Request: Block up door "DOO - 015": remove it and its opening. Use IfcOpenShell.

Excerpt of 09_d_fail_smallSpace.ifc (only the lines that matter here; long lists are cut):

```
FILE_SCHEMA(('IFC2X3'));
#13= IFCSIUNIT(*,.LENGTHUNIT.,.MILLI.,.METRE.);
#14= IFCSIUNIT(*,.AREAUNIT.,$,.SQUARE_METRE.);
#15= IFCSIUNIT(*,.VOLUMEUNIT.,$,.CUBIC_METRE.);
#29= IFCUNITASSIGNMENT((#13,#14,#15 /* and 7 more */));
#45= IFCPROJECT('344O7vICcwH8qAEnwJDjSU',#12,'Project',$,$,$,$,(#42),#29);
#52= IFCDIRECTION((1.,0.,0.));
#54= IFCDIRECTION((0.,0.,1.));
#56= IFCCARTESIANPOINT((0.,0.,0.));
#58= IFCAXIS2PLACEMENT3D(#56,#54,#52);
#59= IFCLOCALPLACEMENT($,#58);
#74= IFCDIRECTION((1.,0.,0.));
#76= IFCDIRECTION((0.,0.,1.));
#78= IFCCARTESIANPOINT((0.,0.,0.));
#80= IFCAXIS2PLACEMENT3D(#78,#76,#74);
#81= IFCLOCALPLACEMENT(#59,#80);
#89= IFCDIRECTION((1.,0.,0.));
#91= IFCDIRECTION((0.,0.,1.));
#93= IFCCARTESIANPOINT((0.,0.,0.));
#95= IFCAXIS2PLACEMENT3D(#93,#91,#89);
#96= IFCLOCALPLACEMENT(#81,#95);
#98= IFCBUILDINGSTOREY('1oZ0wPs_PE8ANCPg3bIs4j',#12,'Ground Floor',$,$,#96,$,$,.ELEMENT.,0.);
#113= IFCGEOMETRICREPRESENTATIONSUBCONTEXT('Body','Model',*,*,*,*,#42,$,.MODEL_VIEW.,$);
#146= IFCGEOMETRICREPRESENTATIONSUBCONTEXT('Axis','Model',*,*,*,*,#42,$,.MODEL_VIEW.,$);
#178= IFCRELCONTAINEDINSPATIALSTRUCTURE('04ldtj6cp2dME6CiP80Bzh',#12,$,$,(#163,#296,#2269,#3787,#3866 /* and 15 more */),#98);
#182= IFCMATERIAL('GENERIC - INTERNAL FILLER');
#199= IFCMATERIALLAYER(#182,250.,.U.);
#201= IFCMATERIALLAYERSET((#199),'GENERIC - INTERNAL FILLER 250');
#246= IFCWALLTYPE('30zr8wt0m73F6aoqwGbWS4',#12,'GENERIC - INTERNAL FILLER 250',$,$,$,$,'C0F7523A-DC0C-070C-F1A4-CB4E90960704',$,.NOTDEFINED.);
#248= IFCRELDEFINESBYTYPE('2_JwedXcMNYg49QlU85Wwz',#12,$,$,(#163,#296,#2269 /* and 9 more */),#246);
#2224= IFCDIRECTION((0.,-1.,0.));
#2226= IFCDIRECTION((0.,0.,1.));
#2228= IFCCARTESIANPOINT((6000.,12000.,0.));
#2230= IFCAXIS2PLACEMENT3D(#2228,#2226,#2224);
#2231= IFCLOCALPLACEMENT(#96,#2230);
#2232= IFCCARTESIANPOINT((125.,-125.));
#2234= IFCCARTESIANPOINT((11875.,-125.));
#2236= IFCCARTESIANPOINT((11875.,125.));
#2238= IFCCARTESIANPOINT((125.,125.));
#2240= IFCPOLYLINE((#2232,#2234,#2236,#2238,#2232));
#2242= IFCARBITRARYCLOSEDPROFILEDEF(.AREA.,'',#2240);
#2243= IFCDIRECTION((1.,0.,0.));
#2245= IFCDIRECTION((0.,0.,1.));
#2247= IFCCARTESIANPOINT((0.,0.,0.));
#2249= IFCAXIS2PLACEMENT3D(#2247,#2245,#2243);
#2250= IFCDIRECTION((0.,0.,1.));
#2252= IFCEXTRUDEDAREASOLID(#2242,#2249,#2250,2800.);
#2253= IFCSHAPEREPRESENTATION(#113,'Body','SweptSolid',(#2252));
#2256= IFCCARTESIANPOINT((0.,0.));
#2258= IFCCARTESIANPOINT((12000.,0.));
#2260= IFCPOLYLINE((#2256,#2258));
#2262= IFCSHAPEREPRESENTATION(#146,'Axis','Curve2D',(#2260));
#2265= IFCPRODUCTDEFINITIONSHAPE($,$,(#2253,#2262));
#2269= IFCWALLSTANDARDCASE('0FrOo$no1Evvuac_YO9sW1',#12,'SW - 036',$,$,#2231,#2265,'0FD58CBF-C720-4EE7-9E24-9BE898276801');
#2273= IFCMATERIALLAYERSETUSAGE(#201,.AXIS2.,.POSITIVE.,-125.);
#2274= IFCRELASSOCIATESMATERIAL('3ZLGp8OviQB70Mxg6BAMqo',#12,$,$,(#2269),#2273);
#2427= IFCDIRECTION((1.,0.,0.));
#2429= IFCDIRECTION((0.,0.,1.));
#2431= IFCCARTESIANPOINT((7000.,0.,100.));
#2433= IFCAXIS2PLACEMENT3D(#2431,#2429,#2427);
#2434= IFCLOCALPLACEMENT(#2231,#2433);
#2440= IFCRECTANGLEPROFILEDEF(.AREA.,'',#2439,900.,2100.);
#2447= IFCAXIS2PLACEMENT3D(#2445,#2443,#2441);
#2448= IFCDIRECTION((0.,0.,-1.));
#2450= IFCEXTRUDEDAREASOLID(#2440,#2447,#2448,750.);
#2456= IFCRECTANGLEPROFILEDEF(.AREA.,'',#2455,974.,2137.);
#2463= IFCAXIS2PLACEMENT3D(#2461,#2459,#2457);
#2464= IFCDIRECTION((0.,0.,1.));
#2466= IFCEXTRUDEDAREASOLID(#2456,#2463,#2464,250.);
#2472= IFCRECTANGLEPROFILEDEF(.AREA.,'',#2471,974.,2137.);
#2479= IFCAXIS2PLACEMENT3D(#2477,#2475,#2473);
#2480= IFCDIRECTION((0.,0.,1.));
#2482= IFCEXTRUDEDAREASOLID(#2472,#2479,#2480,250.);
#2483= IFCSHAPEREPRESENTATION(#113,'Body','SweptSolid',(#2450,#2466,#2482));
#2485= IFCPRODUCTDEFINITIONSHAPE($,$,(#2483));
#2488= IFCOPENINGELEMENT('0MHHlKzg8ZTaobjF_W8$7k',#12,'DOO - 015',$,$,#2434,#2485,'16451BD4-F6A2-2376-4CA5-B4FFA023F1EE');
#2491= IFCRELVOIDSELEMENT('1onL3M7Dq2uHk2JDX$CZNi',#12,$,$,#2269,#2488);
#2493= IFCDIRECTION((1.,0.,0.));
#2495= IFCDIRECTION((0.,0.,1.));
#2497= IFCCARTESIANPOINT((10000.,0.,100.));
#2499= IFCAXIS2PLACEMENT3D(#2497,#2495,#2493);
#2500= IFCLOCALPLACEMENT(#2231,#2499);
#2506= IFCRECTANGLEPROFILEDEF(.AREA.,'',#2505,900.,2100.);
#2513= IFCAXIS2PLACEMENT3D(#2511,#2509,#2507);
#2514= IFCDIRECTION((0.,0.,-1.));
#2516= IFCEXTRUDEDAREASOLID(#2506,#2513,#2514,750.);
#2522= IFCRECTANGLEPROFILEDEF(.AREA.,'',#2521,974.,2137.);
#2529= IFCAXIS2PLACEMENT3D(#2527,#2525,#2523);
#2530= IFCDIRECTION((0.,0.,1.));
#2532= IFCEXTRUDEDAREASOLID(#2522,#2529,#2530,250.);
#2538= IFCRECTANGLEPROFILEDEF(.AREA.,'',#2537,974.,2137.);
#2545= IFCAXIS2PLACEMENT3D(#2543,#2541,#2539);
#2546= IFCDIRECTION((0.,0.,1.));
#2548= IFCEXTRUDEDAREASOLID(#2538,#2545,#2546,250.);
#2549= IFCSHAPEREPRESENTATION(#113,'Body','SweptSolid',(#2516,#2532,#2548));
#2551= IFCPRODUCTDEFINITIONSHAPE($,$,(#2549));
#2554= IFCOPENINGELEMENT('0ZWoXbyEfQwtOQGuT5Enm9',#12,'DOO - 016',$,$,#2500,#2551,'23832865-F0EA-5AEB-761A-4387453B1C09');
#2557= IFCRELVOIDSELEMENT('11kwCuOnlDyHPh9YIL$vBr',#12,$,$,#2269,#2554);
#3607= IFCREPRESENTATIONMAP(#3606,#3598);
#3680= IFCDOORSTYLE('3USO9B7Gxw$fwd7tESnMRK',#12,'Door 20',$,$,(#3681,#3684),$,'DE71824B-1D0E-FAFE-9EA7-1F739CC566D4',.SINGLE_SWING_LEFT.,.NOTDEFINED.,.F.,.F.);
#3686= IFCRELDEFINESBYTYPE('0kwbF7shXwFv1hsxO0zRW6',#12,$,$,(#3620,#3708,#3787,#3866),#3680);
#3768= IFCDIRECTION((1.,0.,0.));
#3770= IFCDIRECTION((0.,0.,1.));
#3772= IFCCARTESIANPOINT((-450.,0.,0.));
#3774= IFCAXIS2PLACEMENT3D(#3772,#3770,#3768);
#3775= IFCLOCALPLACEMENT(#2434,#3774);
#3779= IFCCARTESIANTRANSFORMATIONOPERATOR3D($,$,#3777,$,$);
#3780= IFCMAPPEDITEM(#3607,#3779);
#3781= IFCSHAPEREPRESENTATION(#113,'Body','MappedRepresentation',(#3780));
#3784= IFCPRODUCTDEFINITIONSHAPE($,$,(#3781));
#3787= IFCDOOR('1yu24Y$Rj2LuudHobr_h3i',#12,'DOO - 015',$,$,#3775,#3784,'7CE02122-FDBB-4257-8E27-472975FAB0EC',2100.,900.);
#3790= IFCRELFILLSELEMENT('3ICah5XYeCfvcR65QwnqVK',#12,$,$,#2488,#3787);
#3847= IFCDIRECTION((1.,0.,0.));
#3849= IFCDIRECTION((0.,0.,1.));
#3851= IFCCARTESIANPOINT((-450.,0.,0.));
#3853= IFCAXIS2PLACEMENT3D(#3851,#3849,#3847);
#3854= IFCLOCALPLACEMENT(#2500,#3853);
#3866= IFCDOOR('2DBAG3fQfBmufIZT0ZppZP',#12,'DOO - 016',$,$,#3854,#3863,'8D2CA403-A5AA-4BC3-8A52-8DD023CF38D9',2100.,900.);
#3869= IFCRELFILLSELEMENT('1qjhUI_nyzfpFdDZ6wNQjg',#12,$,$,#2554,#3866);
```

```python
import ifcopenshell
import ifcopenshell.api.feature
import ifcopenshell.api.root
import ifcopenshell.geom
import ifcopenshell.util.shape

model = ifcopenshell.open("09_d_fail_smallSpace.ifc")
settings = ifcopenshell.geom.settings()


def volume(element):
    """Net volume in cubic metres, openings subtracted."""
    shape = ifcopenshell.geom.create_shape(settings, element)
    return ifcopenshell.util.shape.get_volume(shape.geometry)


door = model.by_guid("1yu24Y$Rj2LuudHobr_h3i")
opening = door.FillsVoids[0].RelatingOpeningElement
wall = opening.VoidsElements[0].RelatingBuildingElement
before = volume(wall)

ifcopenshell.api.root.remove_product(model, product=door)
ifcopenshell.api.feature.remove_feature(model, feature=opening)

after = volume(wall)

print(f"wall volume {before:.3f} -> {after:.3f} m3")

model.write("09_d_fail_smallSpace_v2.ifc")
```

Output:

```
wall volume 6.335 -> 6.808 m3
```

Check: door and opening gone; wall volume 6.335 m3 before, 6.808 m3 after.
